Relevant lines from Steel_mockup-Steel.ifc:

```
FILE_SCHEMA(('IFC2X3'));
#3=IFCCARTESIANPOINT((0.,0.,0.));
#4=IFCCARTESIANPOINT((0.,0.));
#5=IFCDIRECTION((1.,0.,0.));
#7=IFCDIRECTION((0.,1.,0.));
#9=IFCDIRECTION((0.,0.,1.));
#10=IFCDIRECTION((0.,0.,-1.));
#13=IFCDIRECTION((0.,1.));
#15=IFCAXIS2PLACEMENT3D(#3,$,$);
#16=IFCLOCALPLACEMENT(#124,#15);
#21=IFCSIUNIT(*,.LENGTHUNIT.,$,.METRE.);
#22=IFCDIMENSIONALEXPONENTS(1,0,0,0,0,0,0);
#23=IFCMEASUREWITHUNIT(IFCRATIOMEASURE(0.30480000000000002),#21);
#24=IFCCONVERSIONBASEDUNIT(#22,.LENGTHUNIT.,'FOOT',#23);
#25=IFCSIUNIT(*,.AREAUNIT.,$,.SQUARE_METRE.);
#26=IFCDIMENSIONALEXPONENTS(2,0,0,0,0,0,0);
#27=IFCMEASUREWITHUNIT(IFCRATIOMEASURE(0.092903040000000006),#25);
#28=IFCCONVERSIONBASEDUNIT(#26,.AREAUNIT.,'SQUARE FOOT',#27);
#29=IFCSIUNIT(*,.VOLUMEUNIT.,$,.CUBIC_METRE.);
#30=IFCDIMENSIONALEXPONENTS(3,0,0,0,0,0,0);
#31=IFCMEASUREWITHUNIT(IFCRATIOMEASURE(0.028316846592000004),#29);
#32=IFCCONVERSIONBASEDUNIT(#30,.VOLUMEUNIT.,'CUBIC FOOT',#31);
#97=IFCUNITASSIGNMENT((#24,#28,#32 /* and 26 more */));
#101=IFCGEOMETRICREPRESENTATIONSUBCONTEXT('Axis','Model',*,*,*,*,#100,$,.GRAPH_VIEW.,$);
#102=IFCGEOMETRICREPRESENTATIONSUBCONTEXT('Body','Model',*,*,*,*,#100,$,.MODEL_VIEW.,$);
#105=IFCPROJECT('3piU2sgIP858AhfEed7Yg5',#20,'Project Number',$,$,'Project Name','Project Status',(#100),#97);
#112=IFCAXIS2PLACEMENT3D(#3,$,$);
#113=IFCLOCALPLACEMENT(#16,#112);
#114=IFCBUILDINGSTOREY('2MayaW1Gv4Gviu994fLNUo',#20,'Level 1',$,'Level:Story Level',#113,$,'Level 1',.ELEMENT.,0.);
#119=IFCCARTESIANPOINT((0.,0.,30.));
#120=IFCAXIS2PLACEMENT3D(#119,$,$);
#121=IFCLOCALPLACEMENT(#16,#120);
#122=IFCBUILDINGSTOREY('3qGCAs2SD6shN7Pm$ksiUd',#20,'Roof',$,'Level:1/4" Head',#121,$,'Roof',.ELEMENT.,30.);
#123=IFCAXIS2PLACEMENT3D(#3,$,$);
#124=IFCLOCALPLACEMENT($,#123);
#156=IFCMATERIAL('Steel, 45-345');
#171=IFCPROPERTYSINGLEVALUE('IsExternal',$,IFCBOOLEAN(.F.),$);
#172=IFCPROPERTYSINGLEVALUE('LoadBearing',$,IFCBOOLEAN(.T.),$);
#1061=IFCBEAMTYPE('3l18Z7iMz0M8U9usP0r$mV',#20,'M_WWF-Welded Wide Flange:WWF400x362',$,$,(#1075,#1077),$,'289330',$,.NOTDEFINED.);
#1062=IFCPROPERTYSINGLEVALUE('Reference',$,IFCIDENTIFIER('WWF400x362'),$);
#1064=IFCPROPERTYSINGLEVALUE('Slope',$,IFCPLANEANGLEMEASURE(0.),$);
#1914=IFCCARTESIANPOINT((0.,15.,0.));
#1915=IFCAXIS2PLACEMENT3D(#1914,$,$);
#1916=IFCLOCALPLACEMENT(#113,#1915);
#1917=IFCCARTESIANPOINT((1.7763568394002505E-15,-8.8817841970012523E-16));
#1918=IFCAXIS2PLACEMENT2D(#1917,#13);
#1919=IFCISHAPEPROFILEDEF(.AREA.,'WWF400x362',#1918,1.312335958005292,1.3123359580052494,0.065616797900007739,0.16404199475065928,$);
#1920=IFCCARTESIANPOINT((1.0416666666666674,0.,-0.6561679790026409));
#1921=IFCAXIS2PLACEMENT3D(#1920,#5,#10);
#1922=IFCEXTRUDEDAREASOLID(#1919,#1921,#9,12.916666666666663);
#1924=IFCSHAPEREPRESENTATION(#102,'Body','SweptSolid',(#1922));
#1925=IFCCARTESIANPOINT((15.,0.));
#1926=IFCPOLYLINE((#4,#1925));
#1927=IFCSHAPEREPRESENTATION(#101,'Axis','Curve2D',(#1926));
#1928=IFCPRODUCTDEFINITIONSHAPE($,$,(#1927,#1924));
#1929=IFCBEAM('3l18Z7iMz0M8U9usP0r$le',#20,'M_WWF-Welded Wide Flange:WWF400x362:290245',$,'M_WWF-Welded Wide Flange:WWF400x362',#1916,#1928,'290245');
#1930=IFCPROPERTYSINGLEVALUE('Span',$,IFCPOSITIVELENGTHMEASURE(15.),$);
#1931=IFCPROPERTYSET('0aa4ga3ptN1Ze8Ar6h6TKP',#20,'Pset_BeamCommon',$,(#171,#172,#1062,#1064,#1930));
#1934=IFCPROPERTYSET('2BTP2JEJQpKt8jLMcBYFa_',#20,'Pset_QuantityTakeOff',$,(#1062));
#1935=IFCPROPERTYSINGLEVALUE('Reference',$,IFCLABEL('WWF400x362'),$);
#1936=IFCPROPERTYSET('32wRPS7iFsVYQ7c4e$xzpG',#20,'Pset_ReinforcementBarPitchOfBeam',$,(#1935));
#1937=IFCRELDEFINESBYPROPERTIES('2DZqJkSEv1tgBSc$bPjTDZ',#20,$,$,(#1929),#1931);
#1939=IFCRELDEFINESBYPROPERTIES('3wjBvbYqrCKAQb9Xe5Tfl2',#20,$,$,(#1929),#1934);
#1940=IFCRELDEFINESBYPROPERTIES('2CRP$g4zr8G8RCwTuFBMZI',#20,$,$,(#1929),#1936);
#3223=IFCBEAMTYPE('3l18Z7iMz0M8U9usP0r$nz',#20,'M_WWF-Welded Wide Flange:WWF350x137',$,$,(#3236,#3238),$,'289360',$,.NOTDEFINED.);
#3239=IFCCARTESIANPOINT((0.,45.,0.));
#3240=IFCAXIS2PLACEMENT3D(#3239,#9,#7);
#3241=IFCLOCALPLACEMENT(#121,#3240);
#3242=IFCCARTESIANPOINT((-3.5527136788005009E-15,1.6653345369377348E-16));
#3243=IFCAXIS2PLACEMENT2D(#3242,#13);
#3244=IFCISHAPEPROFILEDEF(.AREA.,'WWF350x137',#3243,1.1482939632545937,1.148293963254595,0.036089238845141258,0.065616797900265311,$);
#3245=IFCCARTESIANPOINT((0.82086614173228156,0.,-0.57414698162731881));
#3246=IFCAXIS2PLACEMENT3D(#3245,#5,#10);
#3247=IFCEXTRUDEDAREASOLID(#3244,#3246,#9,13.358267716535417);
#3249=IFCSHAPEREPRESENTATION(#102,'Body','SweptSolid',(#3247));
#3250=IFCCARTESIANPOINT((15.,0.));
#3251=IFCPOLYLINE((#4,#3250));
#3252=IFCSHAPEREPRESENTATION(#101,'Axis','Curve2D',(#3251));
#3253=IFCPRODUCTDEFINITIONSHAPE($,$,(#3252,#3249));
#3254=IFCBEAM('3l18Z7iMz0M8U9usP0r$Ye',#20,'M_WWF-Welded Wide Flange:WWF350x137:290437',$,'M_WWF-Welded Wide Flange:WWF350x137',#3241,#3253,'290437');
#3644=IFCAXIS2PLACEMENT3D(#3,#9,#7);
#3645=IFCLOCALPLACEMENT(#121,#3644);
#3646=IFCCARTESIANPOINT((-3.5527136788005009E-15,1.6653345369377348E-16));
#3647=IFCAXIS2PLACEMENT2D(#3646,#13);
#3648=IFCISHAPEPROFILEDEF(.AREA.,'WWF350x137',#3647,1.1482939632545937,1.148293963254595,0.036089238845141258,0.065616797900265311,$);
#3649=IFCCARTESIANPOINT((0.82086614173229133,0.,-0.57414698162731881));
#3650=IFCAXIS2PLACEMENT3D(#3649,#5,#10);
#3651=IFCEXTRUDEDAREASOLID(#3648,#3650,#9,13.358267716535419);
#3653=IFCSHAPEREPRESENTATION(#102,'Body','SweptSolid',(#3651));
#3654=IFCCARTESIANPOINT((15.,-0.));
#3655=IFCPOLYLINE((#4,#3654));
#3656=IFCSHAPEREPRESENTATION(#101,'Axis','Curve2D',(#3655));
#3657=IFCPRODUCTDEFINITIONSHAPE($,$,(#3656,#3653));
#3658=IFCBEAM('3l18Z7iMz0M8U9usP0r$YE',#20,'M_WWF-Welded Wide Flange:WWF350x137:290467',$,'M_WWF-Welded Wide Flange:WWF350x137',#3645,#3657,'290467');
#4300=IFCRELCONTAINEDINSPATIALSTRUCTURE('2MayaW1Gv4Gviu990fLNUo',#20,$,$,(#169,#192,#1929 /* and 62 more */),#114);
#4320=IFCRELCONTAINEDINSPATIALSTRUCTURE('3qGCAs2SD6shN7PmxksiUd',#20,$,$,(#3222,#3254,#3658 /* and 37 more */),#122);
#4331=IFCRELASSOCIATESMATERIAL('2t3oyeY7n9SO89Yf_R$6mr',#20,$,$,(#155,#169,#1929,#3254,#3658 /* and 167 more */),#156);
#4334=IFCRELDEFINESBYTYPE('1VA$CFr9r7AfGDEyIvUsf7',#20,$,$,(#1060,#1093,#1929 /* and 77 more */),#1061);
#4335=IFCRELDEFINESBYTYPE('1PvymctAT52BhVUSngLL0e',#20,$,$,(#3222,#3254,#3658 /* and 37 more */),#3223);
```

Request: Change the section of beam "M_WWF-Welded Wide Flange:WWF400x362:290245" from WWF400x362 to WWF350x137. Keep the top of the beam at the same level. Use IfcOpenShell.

```python
import ifcopenshell
import ifcopenshell.api.pset
import ifcopenshell.api.type
import ifcopenshell.util.element
import ifcopenshell.util.representation

model = ifcopenshell.open("Steel_mockup-Steel.ifc")

member = model.by_guid("3l18Z7iMz0M8U9usP0r$le")
source = next(p for p in model.by_type("IfcIShapeProfileDef") if p.ProfileName == "WWF350x137")

body = ifcopenshell.util.representation.get_representation(member, "Model", "Body")
solid = body.Items[0]
old_profile = solid.SweptArea

# Copy the section's sizes but keep this member's own profile position.
profile = ifcopenshell.util.element.copy(model, source)
# Profiles are centred, so shift by half the change in depth to hold the top.
shift = (old_profile.OverallDepth - profile.OverallDepth) / 2
x, y = old_profile.Position.Location.Coordinates
up = (-1.0, 0.0)  # upwards, in the solid's own plane
location = model.createIfcCartesianPoint((x + up[0] * shift, y + up[1] * shift))
profile.Position = model.createIfcAxis2Placement2D(location, old_profile.Position.RefDirection)
solid.SweptArea = profile
if not model.get_total_inverses(old_profile):
    ifcopenshell.util.element.remove_deep2(model, old_profile)

new_type = model.by_guid("3l18Z7iMz0M8U9usP0r$nz")
ifcopenshell.api.type.assign_type(
    model, related_objects=[member], relating_type=new_type, should_map_representations=False
)
member.Name = member.Name.replace("WWF400x362", "WWF350x137")
member.ObjectType = "M_WWF-Welded Wide Flange:WWF350x137"
pset = model.by_id(ifcopenshell.util.element.get_pset(member, "Pset_BeamCommon", should_inherit=False)["id"])
ifcopenshell.api.pset.edit_pset(model, pset=pset, properties={"Reference": "WWF350x137"})
pset = model.by_id(ifcopenshell.util.element.get_pset(member, "Pset_QuantityTakeOff", should_inherit=False)["id"])
ifcopenshell.api.pset.edit_pset(model, pset=pset, properties={"Reference": "WWF350x137"})
pset = model.by_id(ifcopenshell.util.element.get_pset(member, "Pset_ReinforcementBarPitchOfBeam", should_inherit=False)["id"])
ifcopenshell.api.pset.edit_pset(model, pset=pset, properties={"Reference": "WWF350x137"})

print(solid.SweptArea)

model.write("Steel_mockup-Steel_v2.ifc")
```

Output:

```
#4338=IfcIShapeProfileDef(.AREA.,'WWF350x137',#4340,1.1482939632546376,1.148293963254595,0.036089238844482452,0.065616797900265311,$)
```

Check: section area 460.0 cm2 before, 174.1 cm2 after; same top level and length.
